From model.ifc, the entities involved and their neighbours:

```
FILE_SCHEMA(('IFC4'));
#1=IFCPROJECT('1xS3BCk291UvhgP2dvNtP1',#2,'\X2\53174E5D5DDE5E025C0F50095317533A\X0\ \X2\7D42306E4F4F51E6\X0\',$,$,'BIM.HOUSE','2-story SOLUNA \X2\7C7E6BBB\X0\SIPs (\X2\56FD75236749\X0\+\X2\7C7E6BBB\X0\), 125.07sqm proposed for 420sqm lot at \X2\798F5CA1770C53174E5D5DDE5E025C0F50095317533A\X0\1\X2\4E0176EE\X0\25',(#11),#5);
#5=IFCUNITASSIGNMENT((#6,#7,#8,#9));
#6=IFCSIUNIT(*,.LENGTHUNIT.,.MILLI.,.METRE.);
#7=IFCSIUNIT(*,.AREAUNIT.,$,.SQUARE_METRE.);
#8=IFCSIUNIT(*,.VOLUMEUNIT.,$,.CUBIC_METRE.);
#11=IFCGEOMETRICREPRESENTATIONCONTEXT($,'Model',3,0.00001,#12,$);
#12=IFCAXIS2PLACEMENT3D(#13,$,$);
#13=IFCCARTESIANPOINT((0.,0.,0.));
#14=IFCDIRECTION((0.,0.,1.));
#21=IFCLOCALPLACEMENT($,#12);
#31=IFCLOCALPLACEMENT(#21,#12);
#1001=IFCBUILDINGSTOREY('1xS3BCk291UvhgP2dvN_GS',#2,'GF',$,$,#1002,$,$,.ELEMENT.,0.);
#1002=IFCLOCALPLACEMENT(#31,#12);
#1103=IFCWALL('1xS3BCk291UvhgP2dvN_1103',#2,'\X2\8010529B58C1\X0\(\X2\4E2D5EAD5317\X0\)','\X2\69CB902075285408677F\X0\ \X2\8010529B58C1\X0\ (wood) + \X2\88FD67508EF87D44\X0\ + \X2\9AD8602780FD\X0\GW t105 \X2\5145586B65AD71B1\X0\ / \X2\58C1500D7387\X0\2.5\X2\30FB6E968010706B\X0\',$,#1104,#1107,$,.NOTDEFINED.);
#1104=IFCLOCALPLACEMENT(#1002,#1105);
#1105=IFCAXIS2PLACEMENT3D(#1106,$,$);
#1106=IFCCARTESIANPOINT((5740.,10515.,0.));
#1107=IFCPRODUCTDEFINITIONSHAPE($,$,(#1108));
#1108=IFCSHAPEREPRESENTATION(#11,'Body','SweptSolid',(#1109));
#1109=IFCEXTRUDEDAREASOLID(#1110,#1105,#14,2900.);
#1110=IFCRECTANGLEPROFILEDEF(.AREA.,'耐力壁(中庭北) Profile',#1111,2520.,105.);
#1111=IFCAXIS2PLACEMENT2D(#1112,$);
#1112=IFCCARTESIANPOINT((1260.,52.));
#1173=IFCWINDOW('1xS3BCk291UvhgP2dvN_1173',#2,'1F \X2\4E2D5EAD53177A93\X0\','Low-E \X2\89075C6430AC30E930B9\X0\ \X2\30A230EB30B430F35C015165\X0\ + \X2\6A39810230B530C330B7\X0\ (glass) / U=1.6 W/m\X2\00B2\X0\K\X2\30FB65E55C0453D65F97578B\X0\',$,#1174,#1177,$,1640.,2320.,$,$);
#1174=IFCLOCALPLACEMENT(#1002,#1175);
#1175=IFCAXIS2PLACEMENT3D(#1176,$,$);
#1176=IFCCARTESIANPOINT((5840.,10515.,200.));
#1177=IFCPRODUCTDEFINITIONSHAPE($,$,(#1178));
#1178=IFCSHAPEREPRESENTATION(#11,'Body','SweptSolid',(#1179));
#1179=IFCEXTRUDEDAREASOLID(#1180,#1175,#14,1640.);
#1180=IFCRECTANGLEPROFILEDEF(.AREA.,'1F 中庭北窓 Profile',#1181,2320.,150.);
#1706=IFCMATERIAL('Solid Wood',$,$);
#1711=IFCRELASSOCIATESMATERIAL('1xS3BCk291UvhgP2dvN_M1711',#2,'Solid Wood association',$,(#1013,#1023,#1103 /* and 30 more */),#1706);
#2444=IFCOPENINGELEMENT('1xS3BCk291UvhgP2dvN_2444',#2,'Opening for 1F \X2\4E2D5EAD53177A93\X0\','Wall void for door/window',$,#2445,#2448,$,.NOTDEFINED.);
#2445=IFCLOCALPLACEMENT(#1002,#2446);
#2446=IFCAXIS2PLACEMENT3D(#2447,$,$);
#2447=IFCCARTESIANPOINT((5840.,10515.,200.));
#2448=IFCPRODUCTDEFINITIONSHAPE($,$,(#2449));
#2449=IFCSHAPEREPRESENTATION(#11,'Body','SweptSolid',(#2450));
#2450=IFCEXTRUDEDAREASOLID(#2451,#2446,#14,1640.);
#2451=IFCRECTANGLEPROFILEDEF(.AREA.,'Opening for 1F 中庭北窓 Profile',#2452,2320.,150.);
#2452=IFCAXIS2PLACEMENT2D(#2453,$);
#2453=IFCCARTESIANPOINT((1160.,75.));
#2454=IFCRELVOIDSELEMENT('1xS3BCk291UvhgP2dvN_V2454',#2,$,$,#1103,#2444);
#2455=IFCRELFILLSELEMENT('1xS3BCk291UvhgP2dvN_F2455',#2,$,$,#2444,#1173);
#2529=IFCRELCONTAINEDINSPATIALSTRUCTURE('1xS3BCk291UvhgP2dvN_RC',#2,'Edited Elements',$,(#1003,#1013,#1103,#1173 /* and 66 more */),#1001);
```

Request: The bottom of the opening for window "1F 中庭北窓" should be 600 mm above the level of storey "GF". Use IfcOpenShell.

```python
import numpy as np
import ifcopenshell
import ifcopenshell.api.geometry
import ifcopenshell.geom
import ifcopenshell.util.element
import ifcopenshell.util.placement
import ifcopenshell.util.shape
import ifcopenshell.util.unit

model = ifcopenshell.open("model.ifc")
unit_scale = ifcopenshell.util.unit.calculate_unit_scale(model)

window = model.by_id(1173)
opening = window.FillsVoids[0].RelatingOpeningElement
storey = ifcopenshell.util.element.get_container(window, ifc_class="IfcBuildingStorey")
level = ifcopenshell.util.placement.get_local_placement(storey.ObjectPlacement)[2, 3]

# The opening's origin need not be at the sill, so measure its lowest point.
shape = ifcopenshell.geom.create_shape(ifcopenshell.geom.settings(), opening)
bottom = ifcopenshell.util.shape.get_shape_bottom_elevation(shape, shape.geometry) / unit_scale
dz = level + 600.0 - bottom

shift = np.array([0.0, 0.0, dz])
# The window is not placed relative to its opening, so move both.
for product in (opening, window):
    matrix = ifcopenshell.util.placement.get_local_placement(product.ObjectPlacement)
    matrix[:3, 3] += shift
    ifcopenshell.api.geometry.edit_object_placement(model, product=product, matrix=matrix, is_si=False)

print(f"moved by {dz * unit_scale:+.3f} m")

model.write("model_updated.ifc")
```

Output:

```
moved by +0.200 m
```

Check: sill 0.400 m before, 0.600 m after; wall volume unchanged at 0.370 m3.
